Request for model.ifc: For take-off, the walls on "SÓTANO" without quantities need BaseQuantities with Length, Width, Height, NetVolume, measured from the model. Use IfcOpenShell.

First a look at what the model holds.

```python
import ifcopenshell
import ifcopenshell.util.element
import ifcopenshell.util.unit

model = ifcopenshell.open("model.ifc")
print(model.schema)
for unit_type in ("LENGTHUNIT", "AREAUNIT", "VOLUMEUNIT"):
    print(unit_type, ifcopenshell.util.unit.calculate_unit_scale(model, unit_type))
storey = next(s for s in model.by_type("IfcBuildingStorey") if s.Name == "SÓTANO")
walls = [e for e in ifcopenshell.util.element.get_decomposition(storey) if e.is_a("IfcWall")]
for e in sorted(walls, key=lambda e: e.id()):
    print(e.id(), e.is_a(), e.Name, list(ifcopenshell.util.element.get_psets(e, qtos_only=True)), sep=" | ")
```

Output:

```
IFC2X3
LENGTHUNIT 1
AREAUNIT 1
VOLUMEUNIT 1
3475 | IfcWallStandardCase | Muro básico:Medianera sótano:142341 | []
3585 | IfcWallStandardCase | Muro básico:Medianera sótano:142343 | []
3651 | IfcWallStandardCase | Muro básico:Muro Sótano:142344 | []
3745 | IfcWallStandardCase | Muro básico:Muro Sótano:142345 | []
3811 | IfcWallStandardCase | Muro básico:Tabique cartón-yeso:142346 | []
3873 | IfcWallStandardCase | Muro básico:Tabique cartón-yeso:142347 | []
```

```python
import ifcopenshell
import ifcopenshell.api.pset
import ifcopenshell.geom
import ifcopenshell.util.element
import ifcopenshell.util.shape
import ifcopenshell.util.unit

model = ifcopenshell.open("model.ifc")
unit_scale = ifcopenshell.util.unit.calculate_unit_scale(model)
volume_scale = ifcopenshell.util.unit.calculate_unit_scale(model, "VOLUMEUNIT")
settings = ifcopenshell.geom.settings()

storey = next(s for s in model.by_type("IfcBuildingStorey") if s.Name == "SÓTANO")
walls = [e for e in ifcopenshell.util.element.get_decomposition(storey) if e.is_a("IfcWall")]

for e in sorted(walls, key=lambda e: e.id()):
    if ifcopenshell.util.element.get_psets(e, qtos_only=True, should_inherit=False):
        continue
    # Geometry comes back in metres, in the element's own axes.
    shape = ifcopenshell.geom.create_shape(settings, e)
    values = {
        "Length": ifcopenshell.util.shape.get_x(shape.geometry) / unit_scale,
        "Width": ifcopenshell.util.shape.get_y(shape.geometry) / unit_scale,
        "Height": ifcopenshell.util.shape.get_z(shape.geometry) / unit_scale,
        "NetVolume": ifcopenshell.util.shape.get_volume(shape.geometry) / volume_scale,
    }
    qto = ifcopenshell.api.pset.add_qto(model, product=e, name="BaseQuantities")
    ifcopenshell.api.pset.edit_qto(model, qto=qto, properties=values)
    print(e.id(), {k: round(v, 3) for k, v in values.items()})

model.write("model-out.ifc")
```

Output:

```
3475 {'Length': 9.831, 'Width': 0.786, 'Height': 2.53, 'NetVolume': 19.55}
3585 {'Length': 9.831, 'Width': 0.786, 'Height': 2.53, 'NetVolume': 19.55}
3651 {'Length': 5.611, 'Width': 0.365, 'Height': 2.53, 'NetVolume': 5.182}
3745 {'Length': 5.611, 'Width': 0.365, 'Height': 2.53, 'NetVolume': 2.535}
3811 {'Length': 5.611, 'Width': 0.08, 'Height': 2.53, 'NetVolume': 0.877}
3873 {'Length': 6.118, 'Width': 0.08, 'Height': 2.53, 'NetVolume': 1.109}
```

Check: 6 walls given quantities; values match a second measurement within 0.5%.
